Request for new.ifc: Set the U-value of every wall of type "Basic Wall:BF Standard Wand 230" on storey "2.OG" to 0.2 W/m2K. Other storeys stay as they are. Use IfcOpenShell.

First a look at what the model holds.

```python
import ifcopenshell
import ifcopenshell.util.element

model = ifcopenshell.open("new.ifc")
print(model.schema)
storey = next(s for s in model.by_type("IfcBuildingStorey") if s.Name == "2.OG")
walls = [e for e in ifcopenshell.util.element.get_decomposition(storey) if e.is_a("IfcWall")]
seen = {}
for e in walls:
    element_type = ifcopenshell.util.element.get_type(e)
    key = (element_type.Name if element_type != e and element_type else None, ifcopenshell.util.element.get_pset(e, "Pset_WallCommon", "ThermalTransmittance"))
    seen[key] = seen.get(key, 0) + 1
for (name, value), count in sorted(seen.items(), key=str):
    print(count, "x", name, "|", value)
```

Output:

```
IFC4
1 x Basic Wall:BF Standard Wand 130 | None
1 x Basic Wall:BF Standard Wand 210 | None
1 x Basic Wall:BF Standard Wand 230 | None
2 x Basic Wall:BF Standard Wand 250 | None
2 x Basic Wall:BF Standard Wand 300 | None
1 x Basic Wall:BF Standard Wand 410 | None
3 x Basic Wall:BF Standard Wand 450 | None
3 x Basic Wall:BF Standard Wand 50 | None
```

```python
import ifcopenshell
import ifcopenshell.api.pset
import ifcopenshell.util.element

model = ifcopenshell.open("new.ifc")

storey = next(s for s in model.by_type("IfcBuildingStorey") if s.Name == "2.OG")
walls = [e for e in ifcopenshell.util.element.get_decomposition(storey) if e.is_a("IfcWall")]

count = 0
for e in walls:
    element_type = ifcopenshell.util.element.get_type(e)
    if element_type in (None, e) or element_type.Name != "Basic Wall:BF Standard Wand 230":
        continue
    # add_pset returns the element's existing set when there is one.
    pset = ifcopenshell.api.pset.add_pset(model, product=e, name="Pset_WallCommon")
    ifcopenshell.api.pset.edit_pset(model, pset=pset, properties={"ThermalTransmittance": 0.2})
    count += 1

print(count, "walls updated")

model.write("new_v2.ifc")
```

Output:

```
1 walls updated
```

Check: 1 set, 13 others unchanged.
